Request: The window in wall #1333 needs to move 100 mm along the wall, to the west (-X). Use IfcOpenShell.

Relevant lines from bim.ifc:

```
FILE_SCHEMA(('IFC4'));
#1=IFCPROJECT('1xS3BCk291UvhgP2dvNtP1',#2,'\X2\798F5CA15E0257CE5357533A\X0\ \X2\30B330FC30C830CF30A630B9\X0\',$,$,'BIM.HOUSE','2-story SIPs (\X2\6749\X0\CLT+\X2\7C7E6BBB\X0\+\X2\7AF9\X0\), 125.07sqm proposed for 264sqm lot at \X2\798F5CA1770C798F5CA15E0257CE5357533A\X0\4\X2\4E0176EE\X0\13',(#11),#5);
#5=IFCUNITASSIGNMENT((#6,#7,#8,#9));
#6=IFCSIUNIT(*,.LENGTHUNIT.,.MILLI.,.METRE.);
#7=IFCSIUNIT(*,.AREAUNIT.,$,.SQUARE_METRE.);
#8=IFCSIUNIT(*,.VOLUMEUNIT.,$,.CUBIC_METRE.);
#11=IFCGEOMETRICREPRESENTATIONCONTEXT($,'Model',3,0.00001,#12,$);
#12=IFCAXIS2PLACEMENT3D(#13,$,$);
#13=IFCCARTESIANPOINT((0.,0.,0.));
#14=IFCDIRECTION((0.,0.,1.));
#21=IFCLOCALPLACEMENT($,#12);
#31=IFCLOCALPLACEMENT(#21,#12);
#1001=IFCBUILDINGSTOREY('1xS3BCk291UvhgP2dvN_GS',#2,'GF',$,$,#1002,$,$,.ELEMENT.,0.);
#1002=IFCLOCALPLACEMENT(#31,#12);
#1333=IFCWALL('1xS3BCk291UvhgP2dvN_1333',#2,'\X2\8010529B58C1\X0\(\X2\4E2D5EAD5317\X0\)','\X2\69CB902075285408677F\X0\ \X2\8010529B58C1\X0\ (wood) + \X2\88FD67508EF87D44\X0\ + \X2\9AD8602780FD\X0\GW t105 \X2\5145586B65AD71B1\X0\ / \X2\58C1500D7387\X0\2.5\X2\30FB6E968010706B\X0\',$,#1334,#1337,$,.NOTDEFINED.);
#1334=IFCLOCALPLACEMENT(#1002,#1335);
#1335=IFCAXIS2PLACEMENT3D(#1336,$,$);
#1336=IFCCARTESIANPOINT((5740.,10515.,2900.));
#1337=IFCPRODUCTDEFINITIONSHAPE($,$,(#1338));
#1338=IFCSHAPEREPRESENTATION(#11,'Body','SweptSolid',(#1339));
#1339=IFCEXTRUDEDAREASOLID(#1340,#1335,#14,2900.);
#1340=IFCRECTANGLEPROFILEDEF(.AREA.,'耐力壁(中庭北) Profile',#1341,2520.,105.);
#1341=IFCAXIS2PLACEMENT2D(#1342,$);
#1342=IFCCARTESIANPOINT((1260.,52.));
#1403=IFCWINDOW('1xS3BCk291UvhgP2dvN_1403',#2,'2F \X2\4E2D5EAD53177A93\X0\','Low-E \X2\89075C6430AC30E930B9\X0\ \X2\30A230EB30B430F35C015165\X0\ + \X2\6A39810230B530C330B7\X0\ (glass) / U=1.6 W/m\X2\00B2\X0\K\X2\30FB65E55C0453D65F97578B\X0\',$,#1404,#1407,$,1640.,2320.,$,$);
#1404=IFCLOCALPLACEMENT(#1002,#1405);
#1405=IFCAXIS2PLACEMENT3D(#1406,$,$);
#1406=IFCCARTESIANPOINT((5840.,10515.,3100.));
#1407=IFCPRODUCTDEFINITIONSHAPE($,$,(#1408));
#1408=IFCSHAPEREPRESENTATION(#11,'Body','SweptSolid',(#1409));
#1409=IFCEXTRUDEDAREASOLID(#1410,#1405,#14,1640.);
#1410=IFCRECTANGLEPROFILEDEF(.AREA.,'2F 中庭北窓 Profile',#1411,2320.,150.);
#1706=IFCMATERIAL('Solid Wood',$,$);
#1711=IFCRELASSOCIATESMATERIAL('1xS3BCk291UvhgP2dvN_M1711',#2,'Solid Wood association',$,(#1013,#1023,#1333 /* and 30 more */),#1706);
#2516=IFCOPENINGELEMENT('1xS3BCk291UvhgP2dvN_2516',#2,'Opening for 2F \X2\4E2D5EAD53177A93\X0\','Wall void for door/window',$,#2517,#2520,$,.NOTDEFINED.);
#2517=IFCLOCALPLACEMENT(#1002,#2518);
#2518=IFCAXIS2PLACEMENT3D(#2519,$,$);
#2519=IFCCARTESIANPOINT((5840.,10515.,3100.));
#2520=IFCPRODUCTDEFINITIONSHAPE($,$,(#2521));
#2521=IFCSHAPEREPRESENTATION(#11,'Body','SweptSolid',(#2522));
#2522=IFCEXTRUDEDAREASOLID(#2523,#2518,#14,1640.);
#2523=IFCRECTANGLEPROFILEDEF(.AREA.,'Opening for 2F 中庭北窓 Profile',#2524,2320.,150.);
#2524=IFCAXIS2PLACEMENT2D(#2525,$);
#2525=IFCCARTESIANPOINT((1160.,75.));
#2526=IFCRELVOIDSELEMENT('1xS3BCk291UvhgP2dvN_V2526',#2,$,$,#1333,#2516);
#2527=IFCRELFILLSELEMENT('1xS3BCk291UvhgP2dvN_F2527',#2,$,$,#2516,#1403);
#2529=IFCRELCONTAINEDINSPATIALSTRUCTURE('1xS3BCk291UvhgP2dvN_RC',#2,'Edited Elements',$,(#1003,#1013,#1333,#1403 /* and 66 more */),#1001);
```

```python
import ifcopenshell
import ifcopenshell.api.geometry
import ifcopenshell.util.placement

model = ifcopenshell.open("bim.ifc")

window = model.by_id(1403)
opening = window.FillsVoids[0].RelatingOpeningElement
wall = opening.VoidsElements[0].RelatingBuildingElement

wall_matrix = ifcopenshell.util.placement.get_local_placement(wall.ObjectPlacement)
shift = wall_matrix[:3, 0] * -100.0
before = ifcopenshell.util.placement.get_local_placement(window.ObjectPlacement)[:3, 3].copy()

# The window is not placed relative to its opening, so move both.
for product in (opening, window):
    matrix = ifcopenshell.util.placement.get_local_placement(product.ObjectPlacement)
    matrix[:3, 3] += shift
    ifcopenshell.api.geometry.edit_object_placement(model, product=product, matrix=matrix, is_si=False)

after = ifcopenshell.util.placement.get_local_placement(window.ObjectPlacement)[:3, 3]
print("window moved by", (after - before).round(3) + 0.0)

model.write("bim-out.ifc")
```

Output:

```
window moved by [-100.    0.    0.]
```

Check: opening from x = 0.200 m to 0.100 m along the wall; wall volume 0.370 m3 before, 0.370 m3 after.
